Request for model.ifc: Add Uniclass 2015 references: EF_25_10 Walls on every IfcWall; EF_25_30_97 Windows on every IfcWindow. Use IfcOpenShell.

First a look at what the model holds.

```python
import ifcopenshell

model = ifcopenshell.open("model.ifc")
print(model.schema)
print("classifications:", [c.Name for c in model.by_type("IfcClassification")])
for ifc_class in ("IfcDoor", "IfcRoof", "IfcStair", "IfcWall", "IfcWindow"):
    print(ifc_class, len(model.by_type(ifc_class)))
```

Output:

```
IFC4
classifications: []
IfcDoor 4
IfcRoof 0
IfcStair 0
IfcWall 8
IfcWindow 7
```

```python
import ifcopenshell
import ifcopenshell.api.classification

model = ifcopenshell.open("model.ifc")

system = ifcopenshell.api.classification.add_classification(model, classification="Uniclass 2015")

codes = {
    "IfcWall": ("EF_25_10", "Walls"),
    "IfcWindow": ("EF_25_30_97", "Windows"),
}
for ifc_class, (code, name) in codes.items():
    products = model.by_type(ifc_class)
    ifcopenshell.api.classification.add_reference(
        model, products=products, classification=system, identification=code, name=name
    )
    print(code, len(products))

model.write("model_edited.ifc")
```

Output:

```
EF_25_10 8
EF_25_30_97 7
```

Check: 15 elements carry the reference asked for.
